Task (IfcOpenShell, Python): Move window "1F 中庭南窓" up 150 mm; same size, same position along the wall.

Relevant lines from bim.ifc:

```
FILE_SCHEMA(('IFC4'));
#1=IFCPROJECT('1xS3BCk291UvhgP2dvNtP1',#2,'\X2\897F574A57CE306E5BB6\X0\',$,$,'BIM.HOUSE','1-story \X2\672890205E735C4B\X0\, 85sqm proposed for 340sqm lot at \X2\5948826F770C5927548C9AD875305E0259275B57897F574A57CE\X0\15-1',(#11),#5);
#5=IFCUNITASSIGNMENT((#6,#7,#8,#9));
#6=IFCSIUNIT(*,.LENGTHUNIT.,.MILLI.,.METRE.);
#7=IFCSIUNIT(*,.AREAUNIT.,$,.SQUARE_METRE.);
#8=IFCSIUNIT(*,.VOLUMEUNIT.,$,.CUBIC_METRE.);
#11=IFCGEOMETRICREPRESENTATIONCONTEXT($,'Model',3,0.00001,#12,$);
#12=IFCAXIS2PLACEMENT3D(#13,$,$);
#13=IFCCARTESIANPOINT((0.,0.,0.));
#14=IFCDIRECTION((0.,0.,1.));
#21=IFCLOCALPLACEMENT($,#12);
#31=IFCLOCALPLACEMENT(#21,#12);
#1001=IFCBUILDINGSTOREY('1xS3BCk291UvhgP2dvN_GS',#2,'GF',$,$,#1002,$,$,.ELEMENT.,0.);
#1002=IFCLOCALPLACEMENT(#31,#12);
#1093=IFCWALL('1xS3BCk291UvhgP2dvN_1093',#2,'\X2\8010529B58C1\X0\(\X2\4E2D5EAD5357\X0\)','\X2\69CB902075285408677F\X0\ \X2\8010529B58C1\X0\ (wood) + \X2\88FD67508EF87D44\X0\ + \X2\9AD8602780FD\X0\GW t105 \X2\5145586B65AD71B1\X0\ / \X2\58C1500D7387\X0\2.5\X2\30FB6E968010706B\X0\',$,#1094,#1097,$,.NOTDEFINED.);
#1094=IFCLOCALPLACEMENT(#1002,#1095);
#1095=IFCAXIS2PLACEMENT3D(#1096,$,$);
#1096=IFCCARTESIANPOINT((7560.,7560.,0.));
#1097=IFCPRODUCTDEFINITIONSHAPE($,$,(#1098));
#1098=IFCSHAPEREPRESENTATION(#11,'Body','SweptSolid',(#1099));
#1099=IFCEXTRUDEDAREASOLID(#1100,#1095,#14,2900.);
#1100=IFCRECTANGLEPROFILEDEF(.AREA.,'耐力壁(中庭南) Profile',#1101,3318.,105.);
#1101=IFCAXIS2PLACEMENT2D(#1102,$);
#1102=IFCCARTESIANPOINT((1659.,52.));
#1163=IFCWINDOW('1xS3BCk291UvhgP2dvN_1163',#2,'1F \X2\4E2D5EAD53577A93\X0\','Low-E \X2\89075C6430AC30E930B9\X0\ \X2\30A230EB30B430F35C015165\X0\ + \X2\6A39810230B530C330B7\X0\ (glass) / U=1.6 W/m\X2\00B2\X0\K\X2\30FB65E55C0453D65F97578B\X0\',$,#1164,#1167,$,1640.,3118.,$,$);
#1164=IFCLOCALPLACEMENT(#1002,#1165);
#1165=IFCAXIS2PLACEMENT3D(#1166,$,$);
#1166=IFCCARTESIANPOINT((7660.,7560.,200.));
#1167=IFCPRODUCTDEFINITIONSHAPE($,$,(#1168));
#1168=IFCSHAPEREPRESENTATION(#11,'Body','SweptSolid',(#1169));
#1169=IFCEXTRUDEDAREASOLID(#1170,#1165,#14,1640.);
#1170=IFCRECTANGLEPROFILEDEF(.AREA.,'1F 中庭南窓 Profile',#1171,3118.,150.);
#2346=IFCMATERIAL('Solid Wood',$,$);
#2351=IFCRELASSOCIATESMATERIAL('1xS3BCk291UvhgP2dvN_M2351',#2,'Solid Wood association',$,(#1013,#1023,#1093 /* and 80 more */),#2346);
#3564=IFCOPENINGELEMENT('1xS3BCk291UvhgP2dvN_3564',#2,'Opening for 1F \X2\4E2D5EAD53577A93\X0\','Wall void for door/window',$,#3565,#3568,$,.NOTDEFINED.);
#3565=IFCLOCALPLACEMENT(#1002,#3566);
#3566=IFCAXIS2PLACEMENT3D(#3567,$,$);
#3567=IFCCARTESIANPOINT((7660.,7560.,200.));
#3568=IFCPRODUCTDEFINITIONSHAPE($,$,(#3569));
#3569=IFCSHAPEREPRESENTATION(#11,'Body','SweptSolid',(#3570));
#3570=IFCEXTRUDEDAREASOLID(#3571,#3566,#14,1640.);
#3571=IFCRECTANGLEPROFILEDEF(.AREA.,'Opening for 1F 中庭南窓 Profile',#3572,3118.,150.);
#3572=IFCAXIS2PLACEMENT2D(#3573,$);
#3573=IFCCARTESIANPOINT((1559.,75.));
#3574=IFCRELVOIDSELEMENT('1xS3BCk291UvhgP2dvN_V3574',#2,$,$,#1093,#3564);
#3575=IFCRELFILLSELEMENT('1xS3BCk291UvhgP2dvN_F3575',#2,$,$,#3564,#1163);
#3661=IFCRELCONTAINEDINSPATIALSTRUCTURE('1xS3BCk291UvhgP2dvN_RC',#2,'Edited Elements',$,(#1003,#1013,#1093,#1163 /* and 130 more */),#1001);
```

```python
import numpy as np
import ifcopenshell
import ifcopenshell.api.geometry
import ifcopenshell.util.placement
import ifcopenshell.util.unit

model = ifcopenshell.open("bim.ifc")
unit_scale = ifcopenshell.util.unit.calculate_unit_scale(model)

window = model.by_guid("1xS3BCk291UvhgP2dvN_1163")
opening = window.FillsVoids[0].RelatingOpeningElement
dz = 0.15 / unit_scale

shift = np.array([0.0, 0.0, dz])
# The window is not placed relative to its opening, so move both.
for product in (opening, window):
    matrix = ifcopenshell.util.placement.get_local_placement(product.ObjectPlacement)
    matrix[:3, 3] += shift
    ifcopenshell.api.geometry.edit_object_placement(model, product=product, matrix=matrix, is_si=False)

print(f"moved by {dz * unit_scale:+.3f} m")

model.write("bim_updated.ifc")
```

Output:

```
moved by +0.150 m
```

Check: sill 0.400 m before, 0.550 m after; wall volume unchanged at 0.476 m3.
